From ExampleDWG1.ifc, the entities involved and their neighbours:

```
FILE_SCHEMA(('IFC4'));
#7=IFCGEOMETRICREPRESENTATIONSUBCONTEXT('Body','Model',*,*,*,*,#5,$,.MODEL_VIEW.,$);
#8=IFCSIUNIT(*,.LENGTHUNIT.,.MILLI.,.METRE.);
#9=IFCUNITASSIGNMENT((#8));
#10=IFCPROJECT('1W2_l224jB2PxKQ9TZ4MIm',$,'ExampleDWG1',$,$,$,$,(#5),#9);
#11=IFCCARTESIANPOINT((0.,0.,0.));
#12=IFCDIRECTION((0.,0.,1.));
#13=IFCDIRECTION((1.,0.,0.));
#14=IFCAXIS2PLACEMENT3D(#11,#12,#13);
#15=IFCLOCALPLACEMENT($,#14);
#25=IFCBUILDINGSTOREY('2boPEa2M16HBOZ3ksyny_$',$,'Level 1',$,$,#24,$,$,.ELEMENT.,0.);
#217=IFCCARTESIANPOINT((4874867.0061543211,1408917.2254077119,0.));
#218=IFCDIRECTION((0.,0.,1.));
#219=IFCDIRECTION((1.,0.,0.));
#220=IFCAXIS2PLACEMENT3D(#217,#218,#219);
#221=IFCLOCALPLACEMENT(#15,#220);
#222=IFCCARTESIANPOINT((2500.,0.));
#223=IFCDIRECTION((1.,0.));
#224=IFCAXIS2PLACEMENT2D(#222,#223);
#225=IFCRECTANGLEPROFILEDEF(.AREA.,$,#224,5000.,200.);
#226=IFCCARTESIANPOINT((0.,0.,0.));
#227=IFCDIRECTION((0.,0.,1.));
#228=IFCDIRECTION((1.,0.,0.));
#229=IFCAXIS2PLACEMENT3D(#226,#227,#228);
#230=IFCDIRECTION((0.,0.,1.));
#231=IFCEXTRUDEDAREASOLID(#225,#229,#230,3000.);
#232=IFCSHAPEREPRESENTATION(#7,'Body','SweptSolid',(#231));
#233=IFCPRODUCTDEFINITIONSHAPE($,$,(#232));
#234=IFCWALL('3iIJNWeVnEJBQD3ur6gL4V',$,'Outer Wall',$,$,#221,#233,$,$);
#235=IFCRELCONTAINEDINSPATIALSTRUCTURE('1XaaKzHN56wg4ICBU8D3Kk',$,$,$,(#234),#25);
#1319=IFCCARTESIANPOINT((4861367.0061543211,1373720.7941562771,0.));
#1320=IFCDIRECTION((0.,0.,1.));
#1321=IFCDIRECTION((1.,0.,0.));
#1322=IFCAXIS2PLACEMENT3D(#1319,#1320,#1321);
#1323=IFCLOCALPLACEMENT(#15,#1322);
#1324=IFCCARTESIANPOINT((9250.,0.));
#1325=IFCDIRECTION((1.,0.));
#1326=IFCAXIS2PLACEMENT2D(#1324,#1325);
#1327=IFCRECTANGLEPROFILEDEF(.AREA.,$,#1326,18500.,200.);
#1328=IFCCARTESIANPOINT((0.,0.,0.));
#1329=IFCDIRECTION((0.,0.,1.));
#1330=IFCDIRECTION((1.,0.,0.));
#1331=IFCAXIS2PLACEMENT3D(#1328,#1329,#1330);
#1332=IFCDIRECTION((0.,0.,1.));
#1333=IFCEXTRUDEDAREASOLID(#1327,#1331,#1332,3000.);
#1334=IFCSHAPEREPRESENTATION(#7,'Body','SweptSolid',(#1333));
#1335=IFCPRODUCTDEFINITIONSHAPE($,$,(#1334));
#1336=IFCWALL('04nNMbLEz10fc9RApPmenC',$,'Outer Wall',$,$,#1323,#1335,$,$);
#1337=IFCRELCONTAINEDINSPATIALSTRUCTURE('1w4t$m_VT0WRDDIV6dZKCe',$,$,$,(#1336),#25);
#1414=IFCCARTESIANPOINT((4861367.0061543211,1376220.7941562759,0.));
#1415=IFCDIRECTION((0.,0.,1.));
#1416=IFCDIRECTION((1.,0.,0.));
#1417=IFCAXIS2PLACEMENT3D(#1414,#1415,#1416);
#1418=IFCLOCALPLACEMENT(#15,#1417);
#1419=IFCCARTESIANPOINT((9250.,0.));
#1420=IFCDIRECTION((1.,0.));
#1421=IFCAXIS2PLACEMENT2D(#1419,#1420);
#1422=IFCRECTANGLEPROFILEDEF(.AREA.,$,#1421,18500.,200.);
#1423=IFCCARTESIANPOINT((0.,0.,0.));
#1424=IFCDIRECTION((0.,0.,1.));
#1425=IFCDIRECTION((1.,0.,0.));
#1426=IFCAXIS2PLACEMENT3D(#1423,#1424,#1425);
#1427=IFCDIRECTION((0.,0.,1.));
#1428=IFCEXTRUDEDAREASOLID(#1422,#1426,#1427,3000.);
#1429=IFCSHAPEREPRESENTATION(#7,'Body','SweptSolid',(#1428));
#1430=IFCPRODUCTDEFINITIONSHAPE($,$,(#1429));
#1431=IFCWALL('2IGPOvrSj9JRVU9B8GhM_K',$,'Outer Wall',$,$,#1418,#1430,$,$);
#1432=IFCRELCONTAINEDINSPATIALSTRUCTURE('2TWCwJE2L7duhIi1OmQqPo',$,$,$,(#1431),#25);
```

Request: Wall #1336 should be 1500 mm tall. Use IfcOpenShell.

```python
import ifcopenshell
import ifcopenshell.geom
import ifcopenshell.util.representation
import ifcopenshell.util.shape
import ifcopenshell.util.unit

model = ifcopenshell.open("ExampleDWG1.ifc")
unit_scale = ifcopenshell.util.unit.calculate_unit_scale(model)
settings = ifcopenshell.geom.settings()


def volume(element):
    """Net volume in cubic metres, openings subtracted."""
    shape = ifcopenshell.geom.create_shape(settings, element)
    return ifcopenshell.util.shape.get_volume(shape.geometry)


wall = model.by_id(1336)
before = volume(wall)

body = ifcopenshell.util.representation.get_representation(wall, "Model", "Body")
solid = body.Items[0]
old_height = solid.Depth
solid.Depth = 1.5 / unit_scale
after = volume(wall)

print(f"height {old_height:g} -> {solid.Depth:g}, volume {before:.3f} -> {after:.3f} m3")

model.write("ExampleDWG1_v2.ifc")
```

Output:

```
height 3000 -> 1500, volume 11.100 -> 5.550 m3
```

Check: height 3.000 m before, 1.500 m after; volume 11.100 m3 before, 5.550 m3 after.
